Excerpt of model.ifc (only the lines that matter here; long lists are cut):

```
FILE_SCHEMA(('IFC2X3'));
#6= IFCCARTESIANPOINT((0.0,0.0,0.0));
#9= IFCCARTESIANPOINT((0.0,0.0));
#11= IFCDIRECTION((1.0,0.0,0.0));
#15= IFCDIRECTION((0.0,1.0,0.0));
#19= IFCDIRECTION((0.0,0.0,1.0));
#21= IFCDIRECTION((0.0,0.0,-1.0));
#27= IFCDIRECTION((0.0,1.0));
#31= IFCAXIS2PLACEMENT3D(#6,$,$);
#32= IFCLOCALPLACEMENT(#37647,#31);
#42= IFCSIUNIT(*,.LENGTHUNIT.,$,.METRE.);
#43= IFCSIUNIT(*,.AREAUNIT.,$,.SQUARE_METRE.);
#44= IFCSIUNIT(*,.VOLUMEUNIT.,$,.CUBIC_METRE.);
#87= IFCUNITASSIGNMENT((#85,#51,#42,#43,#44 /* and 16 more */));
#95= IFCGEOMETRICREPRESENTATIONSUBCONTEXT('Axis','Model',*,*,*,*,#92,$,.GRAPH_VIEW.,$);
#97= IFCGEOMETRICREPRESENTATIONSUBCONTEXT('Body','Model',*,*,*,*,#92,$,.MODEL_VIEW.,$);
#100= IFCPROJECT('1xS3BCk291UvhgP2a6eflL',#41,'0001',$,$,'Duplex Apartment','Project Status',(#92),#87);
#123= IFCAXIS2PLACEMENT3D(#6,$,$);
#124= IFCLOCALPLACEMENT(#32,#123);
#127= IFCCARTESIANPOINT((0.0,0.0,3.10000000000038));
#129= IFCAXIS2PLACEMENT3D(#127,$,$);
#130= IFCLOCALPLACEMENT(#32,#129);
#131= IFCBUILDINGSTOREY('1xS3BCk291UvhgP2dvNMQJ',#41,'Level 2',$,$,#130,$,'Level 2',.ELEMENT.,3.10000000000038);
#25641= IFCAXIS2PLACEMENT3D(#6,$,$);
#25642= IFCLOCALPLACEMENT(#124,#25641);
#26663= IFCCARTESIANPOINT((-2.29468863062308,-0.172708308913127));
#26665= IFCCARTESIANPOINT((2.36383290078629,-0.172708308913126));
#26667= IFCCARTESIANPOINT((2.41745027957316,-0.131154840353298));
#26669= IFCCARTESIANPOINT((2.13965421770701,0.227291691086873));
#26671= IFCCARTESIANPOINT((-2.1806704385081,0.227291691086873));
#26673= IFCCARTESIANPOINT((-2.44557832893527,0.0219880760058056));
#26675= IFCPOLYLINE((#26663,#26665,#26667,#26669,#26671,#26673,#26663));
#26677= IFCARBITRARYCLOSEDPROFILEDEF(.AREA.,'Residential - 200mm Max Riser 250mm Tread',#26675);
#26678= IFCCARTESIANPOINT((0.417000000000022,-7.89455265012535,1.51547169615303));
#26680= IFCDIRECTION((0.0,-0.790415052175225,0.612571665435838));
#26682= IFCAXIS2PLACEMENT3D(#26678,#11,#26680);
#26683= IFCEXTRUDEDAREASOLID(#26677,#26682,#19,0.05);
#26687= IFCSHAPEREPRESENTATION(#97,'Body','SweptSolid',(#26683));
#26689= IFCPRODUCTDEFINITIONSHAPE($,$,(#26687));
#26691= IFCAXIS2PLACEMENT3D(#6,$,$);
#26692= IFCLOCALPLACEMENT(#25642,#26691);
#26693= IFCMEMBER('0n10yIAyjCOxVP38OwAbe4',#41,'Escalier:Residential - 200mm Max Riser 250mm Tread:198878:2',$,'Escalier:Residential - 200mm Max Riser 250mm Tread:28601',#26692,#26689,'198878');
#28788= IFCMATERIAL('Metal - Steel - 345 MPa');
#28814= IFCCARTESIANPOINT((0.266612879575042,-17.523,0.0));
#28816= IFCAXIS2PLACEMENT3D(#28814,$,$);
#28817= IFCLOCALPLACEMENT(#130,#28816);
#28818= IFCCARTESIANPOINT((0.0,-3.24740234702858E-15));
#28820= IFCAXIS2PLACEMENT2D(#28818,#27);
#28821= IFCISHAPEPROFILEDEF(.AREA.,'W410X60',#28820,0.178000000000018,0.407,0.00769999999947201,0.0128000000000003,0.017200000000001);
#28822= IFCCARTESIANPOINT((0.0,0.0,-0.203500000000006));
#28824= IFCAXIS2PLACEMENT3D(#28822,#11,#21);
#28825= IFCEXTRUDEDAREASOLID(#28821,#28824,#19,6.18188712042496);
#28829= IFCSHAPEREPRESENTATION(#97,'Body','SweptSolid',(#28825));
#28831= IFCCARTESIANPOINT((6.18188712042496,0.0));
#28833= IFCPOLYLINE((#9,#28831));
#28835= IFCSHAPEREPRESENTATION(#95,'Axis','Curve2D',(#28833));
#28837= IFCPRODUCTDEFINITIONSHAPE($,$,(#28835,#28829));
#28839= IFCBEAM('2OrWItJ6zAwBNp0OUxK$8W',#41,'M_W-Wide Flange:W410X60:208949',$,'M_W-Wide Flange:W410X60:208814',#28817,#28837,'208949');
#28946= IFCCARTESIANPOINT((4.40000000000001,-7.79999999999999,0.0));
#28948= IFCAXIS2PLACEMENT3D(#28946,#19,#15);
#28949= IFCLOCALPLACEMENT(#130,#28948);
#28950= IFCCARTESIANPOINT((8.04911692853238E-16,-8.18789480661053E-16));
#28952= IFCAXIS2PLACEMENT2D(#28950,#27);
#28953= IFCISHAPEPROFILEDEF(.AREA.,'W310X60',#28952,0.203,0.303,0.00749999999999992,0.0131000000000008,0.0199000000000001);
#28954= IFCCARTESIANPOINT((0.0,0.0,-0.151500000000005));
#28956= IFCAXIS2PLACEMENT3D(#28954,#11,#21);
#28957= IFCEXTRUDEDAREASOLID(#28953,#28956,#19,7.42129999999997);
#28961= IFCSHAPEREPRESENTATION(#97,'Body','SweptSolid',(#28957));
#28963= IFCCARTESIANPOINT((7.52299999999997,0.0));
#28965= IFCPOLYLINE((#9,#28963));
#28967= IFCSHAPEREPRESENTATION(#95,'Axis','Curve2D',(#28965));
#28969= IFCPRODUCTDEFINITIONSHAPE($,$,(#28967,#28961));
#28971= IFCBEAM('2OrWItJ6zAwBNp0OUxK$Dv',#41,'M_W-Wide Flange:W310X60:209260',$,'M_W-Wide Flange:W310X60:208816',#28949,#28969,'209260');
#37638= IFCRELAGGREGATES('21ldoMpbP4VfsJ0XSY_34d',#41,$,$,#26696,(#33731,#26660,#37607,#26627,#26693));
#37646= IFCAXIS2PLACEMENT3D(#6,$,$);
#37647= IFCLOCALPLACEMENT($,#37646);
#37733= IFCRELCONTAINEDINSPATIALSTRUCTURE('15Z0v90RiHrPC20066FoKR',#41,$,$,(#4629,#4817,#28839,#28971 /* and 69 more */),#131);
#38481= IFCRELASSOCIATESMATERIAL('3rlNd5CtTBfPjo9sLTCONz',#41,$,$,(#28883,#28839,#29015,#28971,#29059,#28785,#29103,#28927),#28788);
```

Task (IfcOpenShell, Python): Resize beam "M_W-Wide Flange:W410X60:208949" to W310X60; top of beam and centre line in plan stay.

```python
import ifcopenshell
import ifcopenshell.util.element
import ifcopenshell.util.representation

model = ifcopenshell.open("model.ifc")

member = model.by_guid("2OrWItJ6zAwBNp0OUxK$8W")
source = next(p for p in model.by_type("IfcIShapeProfileDef") if p.ProfileName == "W310X60")

body = ifcopenshell.util.representation.get_representation(member, "Model", "Body")
solid = body.Items[0]
old_profile = solid.SweptArea

# Copy the section's sizes but keep this member's own profile position.
profile = ifcopenshell.util.element.copy(model, source)
# Profiles are centred, so shift by half the change in depth to hold the top.
shift = (old_profile.OverallDepth - profile.OverallDepth) / 2
x, y = old_profile.Position.Location.Coordinates
up = (-1.0, 0.0)  # upwards, in the solid's own plane
location = model.createIfcCartesianPoint((x + up[0] * shift, y + up[1] * shift))
profile.Position = model.createIfcAxis2Placement2D(location, old_profile.Position.RefDirection)
solid.SweptArea = profile
if not model.get_total_inverses(old_profile):
    ifcopenshell.util.element.remove_deep2(model, old_profile)
member.Name = member.Name.replace("W410X60", "W310X60")
member.ObjectType = member.ObjectType.replace("W410X60", "W310X60")

print(solid.SweptArea)

model.write("model_rev.ifc")
```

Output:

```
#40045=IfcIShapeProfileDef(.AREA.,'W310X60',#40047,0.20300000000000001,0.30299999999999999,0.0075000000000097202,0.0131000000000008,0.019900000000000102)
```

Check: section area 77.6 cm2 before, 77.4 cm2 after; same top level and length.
